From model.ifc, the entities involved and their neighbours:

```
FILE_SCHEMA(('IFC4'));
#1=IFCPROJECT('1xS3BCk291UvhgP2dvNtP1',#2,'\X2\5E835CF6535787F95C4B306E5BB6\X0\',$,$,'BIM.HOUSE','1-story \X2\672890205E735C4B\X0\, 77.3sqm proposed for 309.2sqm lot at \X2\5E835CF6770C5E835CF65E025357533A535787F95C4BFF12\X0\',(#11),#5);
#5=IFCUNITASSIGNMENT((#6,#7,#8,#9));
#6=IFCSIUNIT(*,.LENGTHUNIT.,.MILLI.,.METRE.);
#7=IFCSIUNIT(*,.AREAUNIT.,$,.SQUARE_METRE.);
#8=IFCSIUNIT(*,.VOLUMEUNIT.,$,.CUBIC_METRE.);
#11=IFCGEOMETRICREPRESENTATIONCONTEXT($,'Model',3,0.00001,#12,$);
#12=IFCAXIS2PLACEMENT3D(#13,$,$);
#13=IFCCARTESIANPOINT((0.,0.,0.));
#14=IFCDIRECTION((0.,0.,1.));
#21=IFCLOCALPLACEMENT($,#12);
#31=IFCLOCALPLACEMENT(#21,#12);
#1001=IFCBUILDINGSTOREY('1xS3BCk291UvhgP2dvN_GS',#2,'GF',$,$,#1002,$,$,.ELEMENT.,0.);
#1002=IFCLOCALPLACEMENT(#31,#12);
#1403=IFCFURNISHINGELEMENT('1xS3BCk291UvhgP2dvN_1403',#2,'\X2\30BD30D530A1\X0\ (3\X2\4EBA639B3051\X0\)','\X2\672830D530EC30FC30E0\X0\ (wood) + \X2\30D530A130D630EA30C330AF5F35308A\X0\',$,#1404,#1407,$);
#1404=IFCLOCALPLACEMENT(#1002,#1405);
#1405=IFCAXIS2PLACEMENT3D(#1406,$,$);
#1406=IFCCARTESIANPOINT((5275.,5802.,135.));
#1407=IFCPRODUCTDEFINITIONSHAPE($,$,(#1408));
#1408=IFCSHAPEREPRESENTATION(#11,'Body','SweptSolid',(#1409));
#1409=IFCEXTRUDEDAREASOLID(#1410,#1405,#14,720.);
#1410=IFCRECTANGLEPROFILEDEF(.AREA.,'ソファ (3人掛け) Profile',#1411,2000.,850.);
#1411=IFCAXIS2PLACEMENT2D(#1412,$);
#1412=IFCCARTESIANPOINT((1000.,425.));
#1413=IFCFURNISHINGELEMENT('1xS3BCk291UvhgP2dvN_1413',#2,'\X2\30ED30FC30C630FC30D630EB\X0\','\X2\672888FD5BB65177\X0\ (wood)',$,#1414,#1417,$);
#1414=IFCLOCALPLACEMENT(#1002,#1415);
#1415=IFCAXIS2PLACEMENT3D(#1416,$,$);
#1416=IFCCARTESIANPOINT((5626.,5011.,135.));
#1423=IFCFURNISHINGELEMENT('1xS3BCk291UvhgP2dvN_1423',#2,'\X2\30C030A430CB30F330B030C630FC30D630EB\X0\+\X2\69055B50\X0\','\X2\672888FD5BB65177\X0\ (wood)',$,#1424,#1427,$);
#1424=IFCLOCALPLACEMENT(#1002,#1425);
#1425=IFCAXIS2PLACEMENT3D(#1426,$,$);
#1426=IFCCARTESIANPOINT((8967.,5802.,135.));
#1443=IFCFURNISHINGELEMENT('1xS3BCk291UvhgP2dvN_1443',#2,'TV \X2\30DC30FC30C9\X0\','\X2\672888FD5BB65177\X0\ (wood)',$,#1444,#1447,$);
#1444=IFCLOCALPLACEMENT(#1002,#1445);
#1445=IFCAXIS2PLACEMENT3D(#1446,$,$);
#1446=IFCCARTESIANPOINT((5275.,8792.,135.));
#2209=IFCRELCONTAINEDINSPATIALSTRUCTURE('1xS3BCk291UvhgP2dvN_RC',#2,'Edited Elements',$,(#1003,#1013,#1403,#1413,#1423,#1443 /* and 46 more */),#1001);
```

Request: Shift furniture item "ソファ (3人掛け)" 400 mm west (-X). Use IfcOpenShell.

```python
import ifcopenshell
import ifcopenshell.api.geometry
import ifcopenshell.util.placement
import ifcopenshell.util.unit

model = ifcopenshell.open("model.ifc")
unit_scale = ifcopenshell.util.unit.calculate_unit_scale(model)

item = model.by_guid("1xS3BCk291UvhgP2dvN_1403")
matrix = ifcopenshell.util.placement.get_local_placement(item.ObjectPlacement)
matrix[0, 3] -= 0.4 / unit_scale
ifcopenshell.api.geometry.edit_object_placement(model, product=item, matrix=matrix, is_si=False)

print(ifcopenshell.util.placement.get_local_placement(item.ObjectPlacement).round(3) + 0.0)

model.write("model_v2.ifc")
```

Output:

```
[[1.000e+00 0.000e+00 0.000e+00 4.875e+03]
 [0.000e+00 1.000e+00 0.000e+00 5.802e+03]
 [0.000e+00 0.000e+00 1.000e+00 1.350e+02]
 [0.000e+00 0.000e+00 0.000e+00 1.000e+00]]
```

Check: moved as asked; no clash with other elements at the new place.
